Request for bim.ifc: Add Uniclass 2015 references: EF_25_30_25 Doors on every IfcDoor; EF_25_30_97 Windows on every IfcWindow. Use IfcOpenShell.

First a look at what the model holds.

```python
import ifcopenshell

model = ifcopenshell.open("bim.ifc")
print(model.schema)
print("classifications:", [c.Name for c in model.by_type("IfcClassification")])
for ifc_class in ("IfcDoor", "IfcRoof", "IfcStair", "IfcWall", "IfcWindow"):
    print(ifc_class, len(model.by_type(ifc_class)))
```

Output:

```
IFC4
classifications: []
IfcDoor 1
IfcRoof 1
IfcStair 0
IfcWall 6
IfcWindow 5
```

```python
import ifcopenshell
import ifcopenshell.api.classification

model = ifcopenshell.open("bim.ifc")

system = ifcopenshell.api.classification.add_classification(model, classification="Uniclass 2015")

codes = {
    "IfcDoor": ("EF_25_30_25", "Doors"),
    "IfcWindow": ("EF_25_30_97", "Windows"),
}
for ifc_class, (code, name) in codes.items():
    products = model.by_type(ifc_class)
    ifcopenshell.api.classification.add_reference(
        model, products=products, classification=system, identification=code, name=name
    )
    print(code, len(products))

model.write("bim_updated.ifc")
```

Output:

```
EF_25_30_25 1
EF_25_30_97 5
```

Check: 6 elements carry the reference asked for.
